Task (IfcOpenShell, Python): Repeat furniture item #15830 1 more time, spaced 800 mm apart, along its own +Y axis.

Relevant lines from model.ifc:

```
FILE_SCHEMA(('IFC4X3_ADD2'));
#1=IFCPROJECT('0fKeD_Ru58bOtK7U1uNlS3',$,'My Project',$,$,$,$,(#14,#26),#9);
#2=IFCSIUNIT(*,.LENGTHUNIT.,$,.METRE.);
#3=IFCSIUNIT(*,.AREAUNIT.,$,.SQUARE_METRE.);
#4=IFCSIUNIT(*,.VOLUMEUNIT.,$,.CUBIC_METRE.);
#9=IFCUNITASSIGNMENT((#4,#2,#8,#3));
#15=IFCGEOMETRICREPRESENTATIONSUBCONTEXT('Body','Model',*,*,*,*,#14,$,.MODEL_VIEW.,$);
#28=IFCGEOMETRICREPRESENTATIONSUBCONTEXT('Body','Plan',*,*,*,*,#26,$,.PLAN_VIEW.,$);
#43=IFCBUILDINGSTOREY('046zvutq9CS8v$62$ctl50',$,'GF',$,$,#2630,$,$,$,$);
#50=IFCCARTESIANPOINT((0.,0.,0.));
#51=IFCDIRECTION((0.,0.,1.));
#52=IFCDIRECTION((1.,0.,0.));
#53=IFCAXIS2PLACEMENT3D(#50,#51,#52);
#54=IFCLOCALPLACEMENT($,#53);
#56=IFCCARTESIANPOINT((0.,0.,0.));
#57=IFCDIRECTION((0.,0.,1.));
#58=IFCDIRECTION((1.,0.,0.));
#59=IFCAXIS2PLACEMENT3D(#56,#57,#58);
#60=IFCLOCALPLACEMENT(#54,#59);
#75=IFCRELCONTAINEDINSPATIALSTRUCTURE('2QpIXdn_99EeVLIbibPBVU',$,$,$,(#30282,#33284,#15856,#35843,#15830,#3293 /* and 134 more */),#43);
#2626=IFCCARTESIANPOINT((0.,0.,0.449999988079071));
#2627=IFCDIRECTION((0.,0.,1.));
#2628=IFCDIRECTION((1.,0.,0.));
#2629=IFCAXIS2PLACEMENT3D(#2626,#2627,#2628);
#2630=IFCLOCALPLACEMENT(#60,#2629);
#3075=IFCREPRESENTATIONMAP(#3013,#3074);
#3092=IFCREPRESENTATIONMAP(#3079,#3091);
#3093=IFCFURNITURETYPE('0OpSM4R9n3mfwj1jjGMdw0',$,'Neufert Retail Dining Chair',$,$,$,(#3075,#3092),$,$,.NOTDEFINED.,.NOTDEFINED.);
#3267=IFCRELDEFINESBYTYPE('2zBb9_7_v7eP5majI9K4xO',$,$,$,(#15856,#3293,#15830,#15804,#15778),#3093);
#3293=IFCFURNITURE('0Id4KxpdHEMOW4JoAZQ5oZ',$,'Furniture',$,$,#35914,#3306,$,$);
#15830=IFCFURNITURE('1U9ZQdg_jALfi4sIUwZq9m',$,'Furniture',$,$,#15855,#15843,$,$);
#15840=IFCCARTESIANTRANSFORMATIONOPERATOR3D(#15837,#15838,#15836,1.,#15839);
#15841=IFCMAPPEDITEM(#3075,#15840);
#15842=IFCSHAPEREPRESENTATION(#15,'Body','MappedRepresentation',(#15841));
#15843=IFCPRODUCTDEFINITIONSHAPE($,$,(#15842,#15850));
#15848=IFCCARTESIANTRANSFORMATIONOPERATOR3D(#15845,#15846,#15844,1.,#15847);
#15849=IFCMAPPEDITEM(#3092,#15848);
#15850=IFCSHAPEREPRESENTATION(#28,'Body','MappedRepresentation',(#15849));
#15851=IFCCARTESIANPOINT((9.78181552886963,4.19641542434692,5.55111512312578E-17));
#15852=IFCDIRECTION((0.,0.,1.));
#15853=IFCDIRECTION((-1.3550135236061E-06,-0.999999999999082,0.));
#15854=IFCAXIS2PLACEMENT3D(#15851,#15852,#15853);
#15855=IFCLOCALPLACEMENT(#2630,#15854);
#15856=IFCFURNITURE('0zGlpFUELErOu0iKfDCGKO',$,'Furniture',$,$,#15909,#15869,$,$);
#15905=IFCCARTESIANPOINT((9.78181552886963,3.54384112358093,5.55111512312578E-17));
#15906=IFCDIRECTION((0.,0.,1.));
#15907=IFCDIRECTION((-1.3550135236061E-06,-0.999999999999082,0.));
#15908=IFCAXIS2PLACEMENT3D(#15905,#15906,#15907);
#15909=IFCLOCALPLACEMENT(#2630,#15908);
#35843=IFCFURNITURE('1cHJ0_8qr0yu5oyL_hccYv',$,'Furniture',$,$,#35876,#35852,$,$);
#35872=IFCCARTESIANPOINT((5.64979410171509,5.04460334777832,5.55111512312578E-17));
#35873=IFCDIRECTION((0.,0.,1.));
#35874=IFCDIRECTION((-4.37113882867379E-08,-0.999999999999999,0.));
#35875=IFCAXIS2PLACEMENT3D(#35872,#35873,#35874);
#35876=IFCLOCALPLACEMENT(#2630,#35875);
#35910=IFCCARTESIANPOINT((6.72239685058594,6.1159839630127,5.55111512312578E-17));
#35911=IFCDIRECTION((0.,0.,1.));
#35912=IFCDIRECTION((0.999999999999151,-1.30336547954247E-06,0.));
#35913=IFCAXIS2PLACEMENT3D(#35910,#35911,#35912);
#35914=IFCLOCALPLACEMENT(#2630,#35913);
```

```python
import ifcopenshell
import ifcopenshell.api.geometry
import ifcopenshell.api.root
import ifcopenshell.util.element
import ifcopenshell.util.placement
import ifcopenshell.util.unit

model = ifcopenshell.open("model.ifc")
unit_scale = ifcopenshell.util.unit.calculate_unit_scale(model)

source = model.by_guid("1U9ZQdg_jALfi4sIUwZq9m")
base = ifcopenshell.util.placement.get_local_placement(source.ObjectPlacement)
step = base[:3, 1] * 0.8 / unit_scale

for i in range(1, 2):
    copy = ifcopenshell.api.root.copy_class(model, product=source)
    copy.Representation = ifcopenshell.util.element.copy_deep(
        model, source.Representation, exclude=["IfcGeometricRepresentationContext", "IfcRepresentationMap"]
    )
    matrix = base.copy()
    matrix[:3, 3] += i * step
    print("added at", matrix[:3, 3].round(3) + 0.0)
    ifcopenshell.api.geometry.edit_object_placement(model, product=copy, matrix=matrix, is_si=False)

model.write("model-out.ifc")
```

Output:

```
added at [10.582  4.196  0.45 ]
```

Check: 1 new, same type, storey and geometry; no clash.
